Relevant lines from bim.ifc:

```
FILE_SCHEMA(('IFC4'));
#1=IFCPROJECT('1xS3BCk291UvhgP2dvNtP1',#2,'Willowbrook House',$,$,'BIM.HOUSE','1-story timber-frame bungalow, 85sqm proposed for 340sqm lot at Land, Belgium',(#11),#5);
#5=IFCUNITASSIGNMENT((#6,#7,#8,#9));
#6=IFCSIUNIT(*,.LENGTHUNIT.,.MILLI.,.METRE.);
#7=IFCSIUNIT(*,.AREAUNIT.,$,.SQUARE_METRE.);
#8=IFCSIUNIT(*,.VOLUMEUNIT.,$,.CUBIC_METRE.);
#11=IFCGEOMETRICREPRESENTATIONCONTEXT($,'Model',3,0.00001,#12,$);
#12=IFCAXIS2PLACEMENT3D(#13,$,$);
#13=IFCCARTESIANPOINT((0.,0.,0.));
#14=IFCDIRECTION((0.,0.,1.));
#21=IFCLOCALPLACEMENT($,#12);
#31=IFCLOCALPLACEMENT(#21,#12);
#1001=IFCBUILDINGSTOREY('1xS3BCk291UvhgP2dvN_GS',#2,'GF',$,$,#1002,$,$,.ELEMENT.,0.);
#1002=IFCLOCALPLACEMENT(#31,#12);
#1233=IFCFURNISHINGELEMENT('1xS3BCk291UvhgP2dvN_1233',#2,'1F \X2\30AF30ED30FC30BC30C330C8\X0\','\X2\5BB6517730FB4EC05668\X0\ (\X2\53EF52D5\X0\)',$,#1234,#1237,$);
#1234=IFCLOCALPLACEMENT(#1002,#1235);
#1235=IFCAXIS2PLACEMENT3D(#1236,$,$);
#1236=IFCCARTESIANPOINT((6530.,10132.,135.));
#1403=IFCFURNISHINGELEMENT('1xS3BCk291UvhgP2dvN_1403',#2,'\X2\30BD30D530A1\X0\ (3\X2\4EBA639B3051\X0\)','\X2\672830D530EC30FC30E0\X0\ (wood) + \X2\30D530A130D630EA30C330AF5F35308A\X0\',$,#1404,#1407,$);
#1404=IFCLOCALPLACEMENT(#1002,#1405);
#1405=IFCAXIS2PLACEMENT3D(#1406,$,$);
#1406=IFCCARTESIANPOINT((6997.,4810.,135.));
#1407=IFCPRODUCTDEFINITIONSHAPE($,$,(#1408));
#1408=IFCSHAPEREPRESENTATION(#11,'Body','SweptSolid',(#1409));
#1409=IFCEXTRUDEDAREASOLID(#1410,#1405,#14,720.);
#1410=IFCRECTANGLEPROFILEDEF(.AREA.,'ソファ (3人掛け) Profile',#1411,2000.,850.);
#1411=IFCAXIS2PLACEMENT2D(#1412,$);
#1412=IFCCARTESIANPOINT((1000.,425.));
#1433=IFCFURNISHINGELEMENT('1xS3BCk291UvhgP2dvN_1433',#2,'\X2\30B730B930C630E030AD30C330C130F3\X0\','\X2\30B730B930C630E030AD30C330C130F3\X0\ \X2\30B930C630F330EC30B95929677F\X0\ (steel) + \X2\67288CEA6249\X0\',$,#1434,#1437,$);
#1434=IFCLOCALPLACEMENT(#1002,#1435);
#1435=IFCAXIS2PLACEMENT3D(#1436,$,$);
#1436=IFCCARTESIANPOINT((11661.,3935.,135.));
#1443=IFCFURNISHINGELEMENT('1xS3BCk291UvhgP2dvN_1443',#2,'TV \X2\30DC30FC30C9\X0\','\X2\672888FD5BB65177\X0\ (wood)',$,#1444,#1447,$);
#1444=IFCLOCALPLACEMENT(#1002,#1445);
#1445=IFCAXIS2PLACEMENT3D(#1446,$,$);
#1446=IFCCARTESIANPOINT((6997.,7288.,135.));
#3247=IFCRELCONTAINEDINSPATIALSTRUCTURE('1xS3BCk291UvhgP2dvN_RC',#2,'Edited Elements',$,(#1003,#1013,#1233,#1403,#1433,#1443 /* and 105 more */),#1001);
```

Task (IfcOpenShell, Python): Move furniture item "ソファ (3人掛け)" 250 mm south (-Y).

```python
import ifcopenshell
import ifcopenshell.api.geometry
import ifcopenshell.util.placement

model = ifcopenshell.open("bim.ifc")

item = model.by_guid("1xS3BCk291UvhgP2dvN_1403")
matrix = ifcopenshell.util.placement.get_local_placement(item.ObjectPlacement)
matrix[1, 3] -= 250.0
ifcopenshell.api.geometry.edit_object_placement(model, product=item, matrix=matrix, is_si=False)

print(ifcopenshell.util.placement.get_local_placement(item.ObjectPlacement).round(3) + 0.0)

model.write("bim-out.ifc")
```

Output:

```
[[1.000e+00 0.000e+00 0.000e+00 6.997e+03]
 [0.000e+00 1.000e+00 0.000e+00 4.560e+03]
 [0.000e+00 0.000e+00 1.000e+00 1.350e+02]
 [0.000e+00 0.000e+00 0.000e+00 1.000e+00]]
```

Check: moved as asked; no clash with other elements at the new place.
